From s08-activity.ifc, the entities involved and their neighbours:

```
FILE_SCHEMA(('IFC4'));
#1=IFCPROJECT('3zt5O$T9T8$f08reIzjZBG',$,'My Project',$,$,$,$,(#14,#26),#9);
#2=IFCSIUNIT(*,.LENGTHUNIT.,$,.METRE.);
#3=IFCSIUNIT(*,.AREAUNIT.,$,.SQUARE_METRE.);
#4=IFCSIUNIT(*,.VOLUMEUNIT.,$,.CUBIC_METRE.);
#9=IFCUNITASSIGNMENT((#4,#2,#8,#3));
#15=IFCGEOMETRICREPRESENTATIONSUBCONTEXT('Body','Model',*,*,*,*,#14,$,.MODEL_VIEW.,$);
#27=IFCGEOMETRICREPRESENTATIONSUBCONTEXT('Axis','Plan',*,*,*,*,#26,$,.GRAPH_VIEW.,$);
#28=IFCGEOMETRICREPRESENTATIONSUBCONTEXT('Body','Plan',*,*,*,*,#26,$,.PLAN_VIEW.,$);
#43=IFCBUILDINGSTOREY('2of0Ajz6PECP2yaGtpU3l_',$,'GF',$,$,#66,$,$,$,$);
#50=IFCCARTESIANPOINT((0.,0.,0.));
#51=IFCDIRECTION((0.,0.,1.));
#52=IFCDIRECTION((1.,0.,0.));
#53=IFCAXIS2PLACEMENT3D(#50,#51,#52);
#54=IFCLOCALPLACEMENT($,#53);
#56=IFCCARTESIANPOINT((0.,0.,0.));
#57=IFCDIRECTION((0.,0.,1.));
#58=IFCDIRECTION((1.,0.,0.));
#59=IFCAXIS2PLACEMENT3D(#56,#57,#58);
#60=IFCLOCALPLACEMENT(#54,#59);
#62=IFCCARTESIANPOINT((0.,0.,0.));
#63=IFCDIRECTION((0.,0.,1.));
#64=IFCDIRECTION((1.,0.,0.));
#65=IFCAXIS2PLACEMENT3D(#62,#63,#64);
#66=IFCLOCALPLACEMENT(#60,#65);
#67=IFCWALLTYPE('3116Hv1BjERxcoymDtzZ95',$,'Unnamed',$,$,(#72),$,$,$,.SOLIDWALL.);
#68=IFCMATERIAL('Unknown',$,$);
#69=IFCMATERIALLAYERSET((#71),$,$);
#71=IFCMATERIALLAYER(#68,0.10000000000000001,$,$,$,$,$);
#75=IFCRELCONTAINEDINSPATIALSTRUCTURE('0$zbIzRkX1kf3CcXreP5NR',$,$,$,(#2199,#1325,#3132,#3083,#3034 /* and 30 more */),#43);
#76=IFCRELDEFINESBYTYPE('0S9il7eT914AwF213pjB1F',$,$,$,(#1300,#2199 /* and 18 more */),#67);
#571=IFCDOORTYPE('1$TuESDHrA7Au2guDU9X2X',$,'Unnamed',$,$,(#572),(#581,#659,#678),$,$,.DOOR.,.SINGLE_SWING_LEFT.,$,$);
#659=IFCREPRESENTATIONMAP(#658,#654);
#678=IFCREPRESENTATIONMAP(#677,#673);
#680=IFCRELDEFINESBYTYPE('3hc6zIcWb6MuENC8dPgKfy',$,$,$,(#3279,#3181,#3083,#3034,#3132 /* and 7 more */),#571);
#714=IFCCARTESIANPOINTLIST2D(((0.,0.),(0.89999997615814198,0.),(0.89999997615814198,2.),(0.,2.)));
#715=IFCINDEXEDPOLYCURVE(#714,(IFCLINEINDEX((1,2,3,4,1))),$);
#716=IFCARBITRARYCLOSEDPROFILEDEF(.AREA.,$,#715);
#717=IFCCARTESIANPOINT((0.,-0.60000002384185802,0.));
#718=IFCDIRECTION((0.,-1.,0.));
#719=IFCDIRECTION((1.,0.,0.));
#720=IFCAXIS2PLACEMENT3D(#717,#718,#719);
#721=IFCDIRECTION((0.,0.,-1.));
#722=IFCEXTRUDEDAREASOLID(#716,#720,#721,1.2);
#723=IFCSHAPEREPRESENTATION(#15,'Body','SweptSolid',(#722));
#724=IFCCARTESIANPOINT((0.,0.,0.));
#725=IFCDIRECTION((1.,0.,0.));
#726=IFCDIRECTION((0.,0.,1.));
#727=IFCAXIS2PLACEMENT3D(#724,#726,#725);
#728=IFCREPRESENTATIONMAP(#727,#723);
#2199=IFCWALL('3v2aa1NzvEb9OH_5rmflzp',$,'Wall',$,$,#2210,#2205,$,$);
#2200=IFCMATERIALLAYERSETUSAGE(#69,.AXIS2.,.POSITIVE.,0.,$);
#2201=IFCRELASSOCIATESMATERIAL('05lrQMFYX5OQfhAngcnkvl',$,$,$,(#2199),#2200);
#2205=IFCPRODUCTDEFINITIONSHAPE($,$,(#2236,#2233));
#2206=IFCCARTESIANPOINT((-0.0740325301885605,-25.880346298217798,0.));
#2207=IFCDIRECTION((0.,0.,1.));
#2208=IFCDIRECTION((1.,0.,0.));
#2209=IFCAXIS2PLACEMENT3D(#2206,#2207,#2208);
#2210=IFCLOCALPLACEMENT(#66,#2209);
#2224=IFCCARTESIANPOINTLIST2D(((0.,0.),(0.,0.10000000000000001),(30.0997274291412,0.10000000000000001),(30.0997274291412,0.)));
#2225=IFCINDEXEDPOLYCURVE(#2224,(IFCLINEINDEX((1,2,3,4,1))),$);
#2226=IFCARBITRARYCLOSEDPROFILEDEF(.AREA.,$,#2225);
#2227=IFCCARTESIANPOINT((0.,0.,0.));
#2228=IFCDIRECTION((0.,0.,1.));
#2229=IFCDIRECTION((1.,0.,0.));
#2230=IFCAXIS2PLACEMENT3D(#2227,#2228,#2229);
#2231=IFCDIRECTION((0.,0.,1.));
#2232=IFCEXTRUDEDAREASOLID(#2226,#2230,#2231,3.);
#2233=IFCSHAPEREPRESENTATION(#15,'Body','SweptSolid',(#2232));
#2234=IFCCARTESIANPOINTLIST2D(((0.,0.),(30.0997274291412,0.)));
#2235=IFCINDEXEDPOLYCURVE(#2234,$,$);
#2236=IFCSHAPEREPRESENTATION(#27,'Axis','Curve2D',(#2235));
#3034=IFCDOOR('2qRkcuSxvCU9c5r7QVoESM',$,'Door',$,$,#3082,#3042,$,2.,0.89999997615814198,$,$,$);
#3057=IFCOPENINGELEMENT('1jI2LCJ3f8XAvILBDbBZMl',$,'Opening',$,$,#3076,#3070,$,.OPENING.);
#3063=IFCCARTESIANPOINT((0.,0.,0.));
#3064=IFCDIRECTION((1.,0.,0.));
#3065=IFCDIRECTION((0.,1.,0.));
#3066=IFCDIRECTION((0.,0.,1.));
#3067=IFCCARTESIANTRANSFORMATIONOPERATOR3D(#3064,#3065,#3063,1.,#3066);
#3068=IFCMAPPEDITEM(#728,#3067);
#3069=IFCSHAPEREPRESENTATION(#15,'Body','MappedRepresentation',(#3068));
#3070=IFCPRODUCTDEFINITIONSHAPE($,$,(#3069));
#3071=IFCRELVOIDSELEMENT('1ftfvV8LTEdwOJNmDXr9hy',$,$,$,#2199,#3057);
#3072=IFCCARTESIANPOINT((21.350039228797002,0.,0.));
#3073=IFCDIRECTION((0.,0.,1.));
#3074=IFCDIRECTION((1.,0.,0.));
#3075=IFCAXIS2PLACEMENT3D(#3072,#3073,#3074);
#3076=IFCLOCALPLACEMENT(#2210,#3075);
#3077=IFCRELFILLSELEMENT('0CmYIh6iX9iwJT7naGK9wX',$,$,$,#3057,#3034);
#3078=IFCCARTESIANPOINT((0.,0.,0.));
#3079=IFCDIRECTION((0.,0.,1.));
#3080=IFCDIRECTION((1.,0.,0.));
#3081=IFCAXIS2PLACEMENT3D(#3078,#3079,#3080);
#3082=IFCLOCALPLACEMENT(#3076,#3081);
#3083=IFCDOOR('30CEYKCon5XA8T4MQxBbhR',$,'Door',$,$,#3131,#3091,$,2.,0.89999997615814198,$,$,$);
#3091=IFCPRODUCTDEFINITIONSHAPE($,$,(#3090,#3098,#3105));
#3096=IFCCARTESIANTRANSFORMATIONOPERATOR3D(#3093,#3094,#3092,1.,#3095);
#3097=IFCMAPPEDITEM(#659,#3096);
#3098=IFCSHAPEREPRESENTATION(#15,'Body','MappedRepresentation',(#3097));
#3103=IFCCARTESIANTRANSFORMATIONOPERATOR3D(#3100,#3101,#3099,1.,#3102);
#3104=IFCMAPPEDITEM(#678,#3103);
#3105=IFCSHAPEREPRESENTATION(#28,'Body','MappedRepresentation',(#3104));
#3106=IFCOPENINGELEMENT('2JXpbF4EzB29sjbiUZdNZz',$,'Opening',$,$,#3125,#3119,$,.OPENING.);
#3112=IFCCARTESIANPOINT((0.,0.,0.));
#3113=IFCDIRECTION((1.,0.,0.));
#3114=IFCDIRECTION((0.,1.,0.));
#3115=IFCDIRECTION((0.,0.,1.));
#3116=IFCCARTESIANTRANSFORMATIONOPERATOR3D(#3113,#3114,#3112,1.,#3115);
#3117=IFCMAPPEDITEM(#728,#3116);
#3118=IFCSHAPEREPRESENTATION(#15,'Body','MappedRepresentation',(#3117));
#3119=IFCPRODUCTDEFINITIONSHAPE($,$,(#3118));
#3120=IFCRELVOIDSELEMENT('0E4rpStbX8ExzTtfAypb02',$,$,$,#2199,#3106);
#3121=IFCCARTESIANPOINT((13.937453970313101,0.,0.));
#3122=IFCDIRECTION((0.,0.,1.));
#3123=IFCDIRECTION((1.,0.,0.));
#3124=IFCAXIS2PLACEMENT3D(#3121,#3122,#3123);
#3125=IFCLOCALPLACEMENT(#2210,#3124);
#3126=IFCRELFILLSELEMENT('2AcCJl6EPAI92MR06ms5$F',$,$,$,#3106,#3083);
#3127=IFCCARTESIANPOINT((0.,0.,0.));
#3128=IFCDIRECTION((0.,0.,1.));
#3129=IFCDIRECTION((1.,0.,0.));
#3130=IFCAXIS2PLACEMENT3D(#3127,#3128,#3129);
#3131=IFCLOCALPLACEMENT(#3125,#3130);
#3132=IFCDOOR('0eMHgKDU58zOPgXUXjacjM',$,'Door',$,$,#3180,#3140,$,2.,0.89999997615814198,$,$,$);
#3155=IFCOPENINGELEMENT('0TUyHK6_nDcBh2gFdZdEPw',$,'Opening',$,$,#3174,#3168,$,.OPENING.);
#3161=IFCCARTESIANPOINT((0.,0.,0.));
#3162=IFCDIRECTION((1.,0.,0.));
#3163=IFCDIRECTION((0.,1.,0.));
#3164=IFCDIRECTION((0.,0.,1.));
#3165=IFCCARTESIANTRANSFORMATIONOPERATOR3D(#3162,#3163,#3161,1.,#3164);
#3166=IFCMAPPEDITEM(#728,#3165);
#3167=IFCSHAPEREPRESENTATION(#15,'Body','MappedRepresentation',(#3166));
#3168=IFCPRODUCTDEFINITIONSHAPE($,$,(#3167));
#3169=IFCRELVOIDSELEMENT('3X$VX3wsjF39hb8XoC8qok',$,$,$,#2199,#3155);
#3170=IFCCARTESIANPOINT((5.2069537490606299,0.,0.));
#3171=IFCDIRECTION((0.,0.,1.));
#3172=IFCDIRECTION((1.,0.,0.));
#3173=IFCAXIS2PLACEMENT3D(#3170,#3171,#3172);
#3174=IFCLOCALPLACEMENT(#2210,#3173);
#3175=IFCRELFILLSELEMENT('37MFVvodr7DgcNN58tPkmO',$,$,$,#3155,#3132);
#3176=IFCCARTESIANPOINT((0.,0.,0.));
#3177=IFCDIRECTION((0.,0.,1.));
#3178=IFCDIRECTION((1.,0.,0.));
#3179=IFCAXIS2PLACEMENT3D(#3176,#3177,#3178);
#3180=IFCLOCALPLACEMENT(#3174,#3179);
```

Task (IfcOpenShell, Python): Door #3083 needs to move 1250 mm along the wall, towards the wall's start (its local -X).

```python
import ifcopenshell
import ifcopenshell.api.geometry
import ifcopenshell.util.placement
import ifcopenshell.util.unit

model = ifcopenshell.open("s08-activity.ifc")
unit_scale = ifcopenshell.util.unit.calculate_unit_scale(model)

door = model.by_guid("30CEYKCon5XA8T4MQxBbhR")
opening = door.FillsVoids[0].RelatingOpeningElement
wall = opening.VoidsElements[0].RelatingBuildingElement

wall_matrix = ifcopenshell.util.placement.get_local_placement(wall.ObjectPlacement)
shift = wall_matrix[:3, 0] * -1.25 / unit_scale
before = ifcopenshell.util.placement.get_local_placement(door.ObjectPlacement)[:3, 3].copy()

# The door is placed relative to its opening, so it follows when the opening moves.
matrix = ifcopenshell.util.placement.get_local_placement(opening.ObjectPlacement)
matrix[:3, 3] += shift
ifcopenshell.api.geometry.edit_object_placement(
    model, product=opening, matrix=matrix, is_si=False, should_transform_children=True
)

after = ifcopenshell.util.placement.get_local_placement(door.ObjectPlacement)[:3, 3]
print("door moved by", (after - before).round(3) + 0.0)

model.write("s08-activity_v2.ifc")
```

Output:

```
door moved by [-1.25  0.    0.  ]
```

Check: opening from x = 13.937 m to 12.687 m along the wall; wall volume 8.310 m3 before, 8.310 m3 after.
